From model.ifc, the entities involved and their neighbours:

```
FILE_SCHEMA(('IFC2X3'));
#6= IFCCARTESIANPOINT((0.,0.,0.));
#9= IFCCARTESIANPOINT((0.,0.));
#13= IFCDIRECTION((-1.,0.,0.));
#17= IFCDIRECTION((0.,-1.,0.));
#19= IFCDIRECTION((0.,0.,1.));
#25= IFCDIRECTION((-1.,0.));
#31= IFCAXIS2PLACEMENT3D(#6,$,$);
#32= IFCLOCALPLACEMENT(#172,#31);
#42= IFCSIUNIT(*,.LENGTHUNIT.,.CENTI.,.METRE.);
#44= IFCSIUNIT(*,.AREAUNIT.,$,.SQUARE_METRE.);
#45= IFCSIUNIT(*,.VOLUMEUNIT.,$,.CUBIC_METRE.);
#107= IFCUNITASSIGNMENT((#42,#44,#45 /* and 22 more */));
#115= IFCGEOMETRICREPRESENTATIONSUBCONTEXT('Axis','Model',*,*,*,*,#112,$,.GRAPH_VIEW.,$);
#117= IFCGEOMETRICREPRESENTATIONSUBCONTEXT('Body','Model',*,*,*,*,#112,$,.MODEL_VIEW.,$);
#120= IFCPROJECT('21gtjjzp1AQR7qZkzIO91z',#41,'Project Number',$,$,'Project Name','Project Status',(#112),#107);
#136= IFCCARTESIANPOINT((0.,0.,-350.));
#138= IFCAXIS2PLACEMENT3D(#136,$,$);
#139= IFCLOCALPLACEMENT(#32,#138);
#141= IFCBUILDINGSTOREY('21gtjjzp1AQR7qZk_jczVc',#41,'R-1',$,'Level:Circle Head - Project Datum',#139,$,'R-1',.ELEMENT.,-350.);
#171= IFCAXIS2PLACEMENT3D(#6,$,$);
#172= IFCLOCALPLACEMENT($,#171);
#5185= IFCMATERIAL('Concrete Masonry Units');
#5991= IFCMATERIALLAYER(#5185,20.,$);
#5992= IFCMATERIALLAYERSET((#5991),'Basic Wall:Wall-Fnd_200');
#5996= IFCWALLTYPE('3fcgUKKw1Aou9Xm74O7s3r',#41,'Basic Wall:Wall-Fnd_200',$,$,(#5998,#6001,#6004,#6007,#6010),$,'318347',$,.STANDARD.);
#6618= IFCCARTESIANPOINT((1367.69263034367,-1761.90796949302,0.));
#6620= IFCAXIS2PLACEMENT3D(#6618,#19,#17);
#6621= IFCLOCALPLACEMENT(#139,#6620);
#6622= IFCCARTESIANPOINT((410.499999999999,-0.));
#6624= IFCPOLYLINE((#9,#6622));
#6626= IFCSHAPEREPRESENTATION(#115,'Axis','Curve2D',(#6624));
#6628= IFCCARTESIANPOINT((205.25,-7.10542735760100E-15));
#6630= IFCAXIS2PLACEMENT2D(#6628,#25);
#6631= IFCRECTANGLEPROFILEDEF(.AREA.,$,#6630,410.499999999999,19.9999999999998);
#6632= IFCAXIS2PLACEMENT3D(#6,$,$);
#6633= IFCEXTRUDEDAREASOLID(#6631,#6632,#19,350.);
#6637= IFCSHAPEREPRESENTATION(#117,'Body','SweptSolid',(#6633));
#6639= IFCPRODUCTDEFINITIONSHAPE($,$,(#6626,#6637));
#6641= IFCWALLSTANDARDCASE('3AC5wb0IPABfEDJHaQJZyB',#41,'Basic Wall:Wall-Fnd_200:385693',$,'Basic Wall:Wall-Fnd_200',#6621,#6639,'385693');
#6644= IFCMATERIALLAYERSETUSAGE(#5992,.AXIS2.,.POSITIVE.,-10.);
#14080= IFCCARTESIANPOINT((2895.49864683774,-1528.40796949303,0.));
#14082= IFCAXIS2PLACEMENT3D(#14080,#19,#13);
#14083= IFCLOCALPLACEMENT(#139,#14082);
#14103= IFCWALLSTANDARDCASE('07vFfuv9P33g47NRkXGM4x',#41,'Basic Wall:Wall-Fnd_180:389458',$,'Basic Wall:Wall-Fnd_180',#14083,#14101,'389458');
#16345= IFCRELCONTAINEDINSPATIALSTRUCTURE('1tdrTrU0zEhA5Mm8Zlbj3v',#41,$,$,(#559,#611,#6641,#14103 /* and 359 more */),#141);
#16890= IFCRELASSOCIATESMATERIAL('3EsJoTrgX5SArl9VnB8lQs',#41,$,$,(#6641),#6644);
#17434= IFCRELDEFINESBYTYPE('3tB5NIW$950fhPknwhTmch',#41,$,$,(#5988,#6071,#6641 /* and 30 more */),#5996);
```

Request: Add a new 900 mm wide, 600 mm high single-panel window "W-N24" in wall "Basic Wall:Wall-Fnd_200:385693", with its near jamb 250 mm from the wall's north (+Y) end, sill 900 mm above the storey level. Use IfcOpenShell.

```python
import numpy as np
import ifcopenshell
import ifcopenshell.api.feature
import ifcopenshell.api.geometry
import ifcopenshell.api.root
import ifcopenshell.api.spatial
import ifcopenshell.api.type
import ifcopenshell.geom
import ifcopenshell.util.element
import ifcopenshell.util.placement
import ifcopenshell.util.representation
import ifcopenshell.util.shape
import ifcopenshell.util.unit

model = ifcopenshell.open("model.ifc")
unit_scale = ifcopenshell.util.unit.calculate_unit_scale(model)
settings = ifcopenshell.geom.settings()


def volume(element):
    """Net volume in cubic metres, openings subtracted."""
    shape = ifcopenshell.geom.create_shape(settings, element)
    return ifcopenshell.util.shape.get_volume(shape.geometry)


wall = model.by_guid("3AC5wb0IPABfEDJHaQJZyB")
storey = ifcopenshell.util.element.get_container(wall, ifc_class="IfcBuildingStorey")
context = ifcopenshell.util.representation.get_context(model, "Model", "Body", "MODEL_VIEW")
before = volume(wall)

width, height, from_end, sill = 0.9, 0.6, 0.25, 0.9  # metres

# The wall runs along its own X axis, and the end named is its -X end.
wall_shape = ifcopenshell.geom.create_shape(settings, wall)
x, y, z = ifcopenshell.util.shape.get_vertices(wall_shape.geometry).T
start = x.min() + from_end
face, thickness = float(y.min()), float(y.max() - y.min())
wall_matrix = ifcopenshell.util.placement.get_local_placement(wall.ObjectPlacement)
level = ifcopenshell.util.placement.get_local_placement(storey.ObjectPlacement)[2, 3]


def in_wall(x, y):
    """Placement at x, y metres in the wall's axes, at sill height."""
    matrix = wall_matrix.copy()
    matrix[:, 3] = wall_matrix @ np.array([x / unit_scale, y / unit_scale, 0.0, 1.0])
    matrix[2, 3] = level + sill / unit_scale
    return matrix


# Opening: a box that overshoots both wall faces by 50 mm.
opening = ifcopenshell.api.root.create_entity(model, ifc_class="IfcOpeningElement")
box = ifcopenshell.api.geometry.add_wall_representation(
    model, context=context, length=width, height=height, thickness=thickness + 0.1
)
ifcopenshell.api.geometry.assign_representation(model, product=opening, representation=box)
ifcopenshell.api.geometry.edit_object_placement(model, product=opening, matrix=in_wall(start, face - 0.05), is_si=False)
ifcopenshell.api.feature.add_feature(model, feature=opening, element=wall)

window = ifcopenshell.api.root.create_entity(model, ifc_class="IfcWindow", name="W-N24")
window.OverallWidth, window.OverallHeight = width / unit_scale, height / unit_scale
body = ifcopenshell.api.geometry.add_window_representation(
    model,
    context=context,
    overall_width=window.OverallWidth,
    overall_height=window.OverallHeight,
    partition_type="SINGLE_PANEL",
)
ifcopenshell.api.geometry.assign_representation(model, product=window, representation=body)
ifcopenshell.api.spatial.assign_container(model, products=[window], relating_structure=storey)
fills = ifcopenshell.api.feature.add_filling(model, opening=opening, element=window)
fills.OwnerHistory = window.OwnerHistory  # required in IFC2X3

# IFC2X3 keeps the operation on the window style.
style = ifcopenshell.api.root.create_entity(model, ifc_class="IfcWindowStyle", name="W-N24")
style.OperationType, style.ConstructionType = "SINGLE_PANEL", "NOTDEFINED"
style.ParameterTakesPrecedence = style.Sizeable = False
ifcopenshell.api.type.assign_type(model, related_objects=[window], relating_type=style)

# Centre the window in the wall's thickness.
ifcopenshell.api.geometry.edit_object_placement(model, product=window, matrix=in_wall(start, face), is_si=False)
window_shape = ifcopenshell.geom.create_shape(settings, window)
depth = ifcopenshell.util.shape.get_vertices(window_shape.geometry)[:, 1]
offset = face + thickness / 2 - (depth.min() + depth.max()) / 2
ifcopenshell.api.geometry.edit_object_placement(model, product=window, matrix=in_wall(start, offset), is_si=False)

after = volume(wall)

print(f"wall volume {before:.3f} -> {after:.3f} m3")

model.write("model-out.ifc")
```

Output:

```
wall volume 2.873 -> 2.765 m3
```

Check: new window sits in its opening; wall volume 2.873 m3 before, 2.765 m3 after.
